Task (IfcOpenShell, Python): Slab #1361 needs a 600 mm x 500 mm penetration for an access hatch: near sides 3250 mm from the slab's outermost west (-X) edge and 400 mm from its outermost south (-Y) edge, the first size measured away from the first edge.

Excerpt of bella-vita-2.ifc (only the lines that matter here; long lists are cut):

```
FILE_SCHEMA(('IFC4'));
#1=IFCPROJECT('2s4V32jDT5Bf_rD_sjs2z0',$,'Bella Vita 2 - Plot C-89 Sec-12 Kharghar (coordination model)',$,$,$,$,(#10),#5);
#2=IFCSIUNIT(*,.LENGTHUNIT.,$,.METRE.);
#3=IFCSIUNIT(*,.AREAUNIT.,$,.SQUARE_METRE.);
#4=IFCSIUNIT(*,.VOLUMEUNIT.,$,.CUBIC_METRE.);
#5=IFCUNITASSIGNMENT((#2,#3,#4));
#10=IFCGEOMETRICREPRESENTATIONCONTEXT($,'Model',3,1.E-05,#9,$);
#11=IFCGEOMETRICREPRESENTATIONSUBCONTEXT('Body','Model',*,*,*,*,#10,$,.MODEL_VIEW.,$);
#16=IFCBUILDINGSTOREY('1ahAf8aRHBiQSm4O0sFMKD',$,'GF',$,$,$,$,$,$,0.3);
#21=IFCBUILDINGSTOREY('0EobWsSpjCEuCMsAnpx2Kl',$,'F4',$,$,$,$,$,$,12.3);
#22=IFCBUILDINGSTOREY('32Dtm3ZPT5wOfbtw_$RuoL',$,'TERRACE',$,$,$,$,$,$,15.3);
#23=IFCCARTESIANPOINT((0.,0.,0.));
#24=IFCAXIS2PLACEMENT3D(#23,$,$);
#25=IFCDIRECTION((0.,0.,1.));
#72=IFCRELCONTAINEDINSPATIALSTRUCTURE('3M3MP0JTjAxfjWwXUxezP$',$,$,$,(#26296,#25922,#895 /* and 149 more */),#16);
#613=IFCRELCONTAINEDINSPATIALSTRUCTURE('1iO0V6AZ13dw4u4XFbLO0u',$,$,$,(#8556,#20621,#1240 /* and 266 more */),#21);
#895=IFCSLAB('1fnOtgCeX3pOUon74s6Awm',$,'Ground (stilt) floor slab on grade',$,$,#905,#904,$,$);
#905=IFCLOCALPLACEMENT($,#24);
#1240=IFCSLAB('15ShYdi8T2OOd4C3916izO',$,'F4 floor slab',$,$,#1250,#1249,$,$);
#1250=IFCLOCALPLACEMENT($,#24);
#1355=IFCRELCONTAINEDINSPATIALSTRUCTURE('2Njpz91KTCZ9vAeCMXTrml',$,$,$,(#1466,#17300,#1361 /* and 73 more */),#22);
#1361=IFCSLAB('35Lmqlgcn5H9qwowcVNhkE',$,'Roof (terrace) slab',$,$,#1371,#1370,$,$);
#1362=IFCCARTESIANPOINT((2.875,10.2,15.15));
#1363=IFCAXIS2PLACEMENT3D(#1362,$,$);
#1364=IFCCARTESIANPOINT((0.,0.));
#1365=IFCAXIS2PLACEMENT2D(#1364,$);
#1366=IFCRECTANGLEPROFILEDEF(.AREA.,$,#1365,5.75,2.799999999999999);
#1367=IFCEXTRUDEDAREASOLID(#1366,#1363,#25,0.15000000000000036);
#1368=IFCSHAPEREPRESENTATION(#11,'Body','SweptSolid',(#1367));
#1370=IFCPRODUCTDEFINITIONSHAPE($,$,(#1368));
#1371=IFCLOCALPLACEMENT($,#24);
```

```python
import numpy as np
import ifcopenshell
import ifcopenshell.api.feature
import ifcopenshell.api.geometry
import ifcopenshell.api.root
import ifcopenshell.geom
import ifcopenshell.util.placement
import ifcopenshell.util.representation
import ifcopenshell.util.shape
import ifcopenshell.util.unit

model = ifcopenshell.open("bella-vita-2.ifc")
unit_scale = ifcopenshell.util.unit.calculate_unit_scale(model)
settings = ifcopenshell.geom.settings()


def volume(element):
    """Net volume in cubic metres, openings subtracted."""
    shape = ifcopenshell.geom.create_shape(settings, element)
    return ifcopenshell.util.shape.get_volume(shape.geometry)


slab = model.by_id(1361)
before = volume(slab)

# Extent in the slab's own axes, in metres. The edges named are its -X and -Y sides.
slab_shape = ifcopenshell.geom.create_shape(settings, slab)
vertices = ifcopenshell.util.shape.get_vertices(slab_shape.geometry)
x_min, y_min, bottom = vertices.min(axis=0)
top = vertices[:, 2].max()

opening = ifcopenshell.api.root.create_entity(model, ifc_class="IfcOpeningElement", name="Access hatch opening", predefined_type="OPENING")
context = ifcopenshell.util.representation.get_context(model, "Model", "Body", "MODEL_VIEW")
width, depth = 0.6, 0.5
outline = [(0.0, 0.0), (width, 0.0), (width, depth), (0.0, depth), (0.0, 0.0)]
# Overshoot both faces by 50 mm so the cut is clean.
shape = ifcopenshell.api.geometry.add_slab_representation(
    model, context=context, depth=top - bottom + 0.1, polyline=outline
)
ifcopenshell.api.geometry.assign_representation(model, product=opening, representation=shape)

matrix = ifcopenshell.util.placement.get_local_placement(slab.ObjectPlacement)
matrix[:, 3] = matrix @ np.append(np.array([x_min + 3.25, y_min + 0.4, bottom - 0.05]) / unit_scale, 1.0)
ifcopenshell.api.geometry.edit_object_placement(model, product=opening, matrix=matrix, is_si=False)
ifcopenshell.api.feature.add_feature(model, feature=opening, element=slab)

after = volume(slab)

print(f"slab volume {before:.3f} -> {after:.3f} m3")

model.write("bella-vita-2-out.ifc")
```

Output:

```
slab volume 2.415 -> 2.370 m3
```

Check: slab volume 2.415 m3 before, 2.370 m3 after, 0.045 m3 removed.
